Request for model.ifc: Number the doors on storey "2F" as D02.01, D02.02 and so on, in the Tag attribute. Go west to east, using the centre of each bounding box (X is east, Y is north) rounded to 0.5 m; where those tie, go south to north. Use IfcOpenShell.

First a look at what the model holds.

```python
import ifcopenshell
import ifcopenshell.util.element
import ifcopenshell.util.placement

model = ifcopenshell.open("model.ifc")
print(model.schema)
storey = next(s for s in model.by_type("IfcBuildingStorey") if s.Name == "2F")
doors = [e for e in ifcopenshell.util.element.get_decomposition(storey) if e.is_a("IfcDoor")]
for e in sorted(doors, key=lambda e: e.id()):
    origin = ifcopenshell.util.placement.get_local_placement(e.ObjectPlacement)[:3, 3]
    print(e.id(), e.Tag, e.Name, origin.round(2) + 0.0, sep=" | ")
```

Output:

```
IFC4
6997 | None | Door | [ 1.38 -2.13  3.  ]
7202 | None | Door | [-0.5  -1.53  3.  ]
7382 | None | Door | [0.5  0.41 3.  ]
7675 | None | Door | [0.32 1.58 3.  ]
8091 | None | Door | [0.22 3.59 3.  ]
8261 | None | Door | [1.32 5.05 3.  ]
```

```python
import ifcopenshell
import ifcopenshell.geom
import ifcopenshell.util.element
import ifcopenshell.util.shape

model = ifcopenshell.open("model.ifc")
settings = ifcopenshell.geom.settings()
settings.set("use-world-coords", True)


def centre(element):
    shape = ifcopenshell.geom.create_shape(settings, element)
    return ifcopenshell.util.shape.get_bbox_centroid(shape.geometry)


storey = next(s for s in model.by_type("IfcBuildingStorey") if s.Name == "2F")
doors = [e for e in ifcopenshell.util.element.get_decomposition(storey) if e.is_a("IfcDoor")]

# Insertion points can sit at a corner or the storey origin, so sort by the geometry (in metres).
centres = {e: centre(e) for e in doors}
doors.sort(key=lambda e: (round(centres[e][0] / 0.5), centres[e][1]))

for i, e in enumerate(doors, start=1):
    number = f"D02.{i:02d}"
    e.Tag = number
    print(e.id(), number)

model.write("model_updated.ifc")
```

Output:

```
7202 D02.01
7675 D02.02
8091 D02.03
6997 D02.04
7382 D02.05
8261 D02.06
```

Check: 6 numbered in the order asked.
